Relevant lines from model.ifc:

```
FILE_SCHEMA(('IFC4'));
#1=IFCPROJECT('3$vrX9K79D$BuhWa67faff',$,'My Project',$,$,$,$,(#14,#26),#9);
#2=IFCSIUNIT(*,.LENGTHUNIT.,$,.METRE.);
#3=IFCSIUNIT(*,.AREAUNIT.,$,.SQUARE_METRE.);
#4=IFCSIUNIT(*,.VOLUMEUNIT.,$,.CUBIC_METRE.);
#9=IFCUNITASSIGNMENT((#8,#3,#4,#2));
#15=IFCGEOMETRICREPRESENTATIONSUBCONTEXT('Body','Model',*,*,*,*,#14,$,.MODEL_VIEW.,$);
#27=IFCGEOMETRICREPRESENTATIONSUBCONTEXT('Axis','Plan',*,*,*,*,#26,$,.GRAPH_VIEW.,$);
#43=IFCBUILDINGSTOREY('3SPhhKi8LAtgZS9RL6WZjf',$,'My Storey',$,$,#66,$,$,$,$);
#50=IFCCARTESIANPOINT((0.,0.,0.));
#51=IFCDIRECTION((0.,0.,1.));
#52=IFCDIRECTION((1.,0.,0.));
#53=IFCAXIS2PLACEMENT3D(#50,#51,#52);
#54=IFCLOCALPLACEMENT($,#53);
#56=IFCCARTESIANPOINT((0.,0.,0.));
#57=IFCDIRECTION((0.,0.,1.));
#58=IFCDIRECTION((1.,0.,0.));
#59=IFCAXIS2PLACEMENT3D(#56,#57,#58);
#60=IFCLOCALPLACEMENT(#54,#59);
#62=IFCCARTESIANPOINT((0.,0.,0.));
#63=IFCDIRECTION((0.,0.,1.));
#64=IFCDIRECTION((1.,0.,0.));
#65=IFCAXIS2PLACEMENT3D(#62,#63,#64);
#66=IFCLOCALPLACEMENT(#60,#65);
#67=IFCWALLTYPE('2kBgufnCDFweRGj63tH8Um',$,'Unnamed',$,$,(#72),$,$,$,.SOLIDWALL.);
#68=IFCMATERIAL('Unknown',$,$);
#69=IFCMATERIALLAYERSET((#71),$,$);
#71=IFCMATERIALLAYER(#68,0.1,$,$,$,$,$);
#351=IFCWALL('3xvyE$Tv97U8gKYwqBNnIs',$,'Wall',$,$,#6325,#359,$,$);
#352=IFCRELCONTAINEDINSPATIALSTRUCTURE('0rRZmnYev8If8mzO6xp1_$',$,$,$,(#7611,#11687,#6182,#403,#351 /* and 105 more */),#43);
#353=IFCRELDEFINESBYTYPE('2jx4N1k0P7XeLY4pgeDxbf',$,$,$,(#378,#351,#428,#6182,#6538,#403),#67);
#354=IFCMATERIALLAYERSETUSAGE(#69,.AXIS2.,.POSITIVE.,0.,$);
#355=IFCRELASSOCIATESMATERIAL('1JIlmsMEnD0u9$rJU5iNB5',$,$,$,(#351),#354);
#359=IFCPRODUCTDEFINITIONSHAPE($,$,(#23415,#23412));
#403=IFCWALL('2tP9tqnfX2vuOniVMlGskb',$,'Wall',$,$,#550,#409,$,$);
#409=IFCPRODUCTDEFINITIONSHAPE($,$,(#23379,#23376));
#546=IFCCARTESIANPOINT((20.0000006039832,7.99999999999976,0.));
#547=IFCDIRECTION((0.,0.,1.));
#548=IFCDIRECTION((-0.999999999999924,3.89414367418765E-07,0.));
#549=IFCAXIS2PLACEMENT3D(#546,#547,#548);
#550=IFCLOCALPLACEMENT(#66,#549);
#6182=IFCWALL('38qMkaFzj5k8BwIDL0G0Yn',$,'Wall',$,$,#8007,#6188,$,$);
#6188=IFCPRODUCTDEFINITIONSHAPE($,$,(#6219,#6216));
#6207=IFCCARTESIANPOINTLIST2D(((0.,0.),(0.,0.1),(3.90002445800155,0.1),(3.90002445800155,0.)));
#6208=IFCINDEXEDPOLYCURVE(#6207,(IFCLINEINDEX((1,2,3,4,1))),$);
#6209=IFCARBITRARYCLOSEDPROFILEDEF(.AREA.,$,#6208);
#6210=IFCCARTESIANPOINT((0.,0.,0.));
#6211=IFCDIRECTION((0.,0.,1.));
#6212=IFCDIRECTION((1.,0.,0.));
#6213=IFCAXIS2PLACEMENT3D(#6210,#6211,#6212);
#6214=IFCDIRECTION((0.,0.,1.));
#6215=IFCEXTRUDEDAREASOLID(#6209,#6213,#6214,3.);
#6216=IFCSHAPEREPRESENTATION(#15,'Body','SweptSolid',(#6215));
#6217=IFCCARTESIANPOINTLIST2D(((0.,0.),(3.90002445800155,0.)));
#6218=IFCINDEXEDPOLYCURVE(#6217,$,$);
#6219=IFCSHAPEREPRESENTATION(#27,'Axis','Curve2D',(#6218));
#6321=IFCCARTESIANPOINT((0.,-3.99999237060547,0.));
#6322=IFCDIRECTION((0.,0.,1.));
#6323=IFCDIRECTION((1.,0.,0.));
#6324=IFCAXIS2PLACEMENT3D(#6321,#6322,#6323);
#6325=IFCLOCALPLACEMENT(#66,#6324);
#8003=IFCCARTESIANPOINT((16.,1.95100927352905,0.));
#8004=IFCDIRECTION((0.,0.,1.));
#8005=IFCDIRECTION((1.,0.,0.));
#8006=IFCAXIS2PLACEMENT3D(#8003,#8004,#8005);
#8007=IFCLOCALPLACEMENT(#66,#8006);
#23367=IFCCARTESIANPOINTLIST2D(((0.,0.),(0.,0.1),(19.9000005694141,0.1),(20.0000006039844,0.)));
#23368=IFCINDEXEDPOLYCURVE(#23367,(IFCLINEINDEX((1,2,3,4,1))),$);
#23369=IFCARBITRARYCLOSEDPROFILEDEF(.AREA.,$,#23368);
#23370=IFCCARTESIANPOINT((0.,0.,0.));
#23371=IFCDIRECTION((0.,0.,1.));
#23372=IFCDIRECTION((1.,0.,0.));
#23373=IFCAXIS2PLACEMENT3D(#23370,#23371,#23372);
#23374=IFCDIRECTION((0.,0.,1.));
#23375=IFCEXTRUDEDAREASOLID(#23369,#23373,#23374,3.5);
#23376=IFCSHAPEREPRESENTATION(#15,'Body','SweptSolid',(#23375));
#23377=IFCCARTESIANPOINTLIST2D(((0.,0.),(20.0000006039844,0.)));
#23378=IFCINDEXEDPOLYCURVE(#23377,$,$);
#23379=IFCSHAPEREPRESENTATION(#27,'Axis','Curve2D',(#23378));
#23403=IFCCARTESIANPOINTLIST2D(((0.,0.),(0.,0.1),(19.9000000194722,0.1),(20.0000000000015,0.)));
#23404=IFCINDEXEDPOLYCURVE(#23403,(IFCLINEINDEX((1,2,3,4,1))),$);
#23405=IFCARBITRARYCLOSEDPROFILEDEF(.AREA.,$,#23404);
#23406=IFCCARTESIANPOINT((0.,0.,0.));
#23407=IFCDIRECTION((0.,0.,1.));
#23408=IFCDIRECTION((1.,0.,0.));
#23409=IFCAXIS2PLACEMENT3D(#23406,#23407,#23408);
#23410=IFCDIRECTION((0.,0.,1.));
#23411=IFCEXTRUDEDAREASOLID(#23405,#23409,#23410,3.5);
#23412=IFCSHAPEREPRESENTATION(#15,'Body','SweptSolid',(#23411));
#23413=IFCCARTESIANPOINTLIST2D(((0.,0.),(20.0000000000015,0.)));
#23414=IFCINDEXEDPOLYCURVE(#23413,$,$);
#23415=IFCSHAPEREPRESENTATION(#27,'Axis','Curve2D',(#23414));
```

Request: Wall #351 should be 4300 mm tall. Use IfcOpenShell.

```python
import ifcopenshell
import ifcopenshell.geom
import ifcopenshell.util.representation
import ifcopenshell.util.shape

model = ifcopenshell.open("model.ifc")
settings = ifcopenshell.geom.settings()


def volume(element):
    """Net volume in cubic metres, openings subtracted."""
    shape = ifcopenshell.geom.create_shape(settings, element)
    return ifcopenshell.util.shape.get_volume(shape.geometry)


wall = model.by_id(351)
before = volume(wall)

body = ifcopenshell.util.representation.get_representation(wall, "Model", "Body")
solid = body.Items[0]
old_height = solid.Depth
solid.Depth = 4.3
after = volume(wall)

print(f"height {old_height:g} -> {solid.Depth:g}, volume {before:.3f} -> {after:.3f} m3")

model.write("model_edited.ifc")
```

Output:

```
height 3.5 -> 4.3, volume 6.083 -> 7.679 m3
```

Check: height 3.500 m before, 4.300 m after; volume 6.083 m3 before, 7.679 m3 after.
